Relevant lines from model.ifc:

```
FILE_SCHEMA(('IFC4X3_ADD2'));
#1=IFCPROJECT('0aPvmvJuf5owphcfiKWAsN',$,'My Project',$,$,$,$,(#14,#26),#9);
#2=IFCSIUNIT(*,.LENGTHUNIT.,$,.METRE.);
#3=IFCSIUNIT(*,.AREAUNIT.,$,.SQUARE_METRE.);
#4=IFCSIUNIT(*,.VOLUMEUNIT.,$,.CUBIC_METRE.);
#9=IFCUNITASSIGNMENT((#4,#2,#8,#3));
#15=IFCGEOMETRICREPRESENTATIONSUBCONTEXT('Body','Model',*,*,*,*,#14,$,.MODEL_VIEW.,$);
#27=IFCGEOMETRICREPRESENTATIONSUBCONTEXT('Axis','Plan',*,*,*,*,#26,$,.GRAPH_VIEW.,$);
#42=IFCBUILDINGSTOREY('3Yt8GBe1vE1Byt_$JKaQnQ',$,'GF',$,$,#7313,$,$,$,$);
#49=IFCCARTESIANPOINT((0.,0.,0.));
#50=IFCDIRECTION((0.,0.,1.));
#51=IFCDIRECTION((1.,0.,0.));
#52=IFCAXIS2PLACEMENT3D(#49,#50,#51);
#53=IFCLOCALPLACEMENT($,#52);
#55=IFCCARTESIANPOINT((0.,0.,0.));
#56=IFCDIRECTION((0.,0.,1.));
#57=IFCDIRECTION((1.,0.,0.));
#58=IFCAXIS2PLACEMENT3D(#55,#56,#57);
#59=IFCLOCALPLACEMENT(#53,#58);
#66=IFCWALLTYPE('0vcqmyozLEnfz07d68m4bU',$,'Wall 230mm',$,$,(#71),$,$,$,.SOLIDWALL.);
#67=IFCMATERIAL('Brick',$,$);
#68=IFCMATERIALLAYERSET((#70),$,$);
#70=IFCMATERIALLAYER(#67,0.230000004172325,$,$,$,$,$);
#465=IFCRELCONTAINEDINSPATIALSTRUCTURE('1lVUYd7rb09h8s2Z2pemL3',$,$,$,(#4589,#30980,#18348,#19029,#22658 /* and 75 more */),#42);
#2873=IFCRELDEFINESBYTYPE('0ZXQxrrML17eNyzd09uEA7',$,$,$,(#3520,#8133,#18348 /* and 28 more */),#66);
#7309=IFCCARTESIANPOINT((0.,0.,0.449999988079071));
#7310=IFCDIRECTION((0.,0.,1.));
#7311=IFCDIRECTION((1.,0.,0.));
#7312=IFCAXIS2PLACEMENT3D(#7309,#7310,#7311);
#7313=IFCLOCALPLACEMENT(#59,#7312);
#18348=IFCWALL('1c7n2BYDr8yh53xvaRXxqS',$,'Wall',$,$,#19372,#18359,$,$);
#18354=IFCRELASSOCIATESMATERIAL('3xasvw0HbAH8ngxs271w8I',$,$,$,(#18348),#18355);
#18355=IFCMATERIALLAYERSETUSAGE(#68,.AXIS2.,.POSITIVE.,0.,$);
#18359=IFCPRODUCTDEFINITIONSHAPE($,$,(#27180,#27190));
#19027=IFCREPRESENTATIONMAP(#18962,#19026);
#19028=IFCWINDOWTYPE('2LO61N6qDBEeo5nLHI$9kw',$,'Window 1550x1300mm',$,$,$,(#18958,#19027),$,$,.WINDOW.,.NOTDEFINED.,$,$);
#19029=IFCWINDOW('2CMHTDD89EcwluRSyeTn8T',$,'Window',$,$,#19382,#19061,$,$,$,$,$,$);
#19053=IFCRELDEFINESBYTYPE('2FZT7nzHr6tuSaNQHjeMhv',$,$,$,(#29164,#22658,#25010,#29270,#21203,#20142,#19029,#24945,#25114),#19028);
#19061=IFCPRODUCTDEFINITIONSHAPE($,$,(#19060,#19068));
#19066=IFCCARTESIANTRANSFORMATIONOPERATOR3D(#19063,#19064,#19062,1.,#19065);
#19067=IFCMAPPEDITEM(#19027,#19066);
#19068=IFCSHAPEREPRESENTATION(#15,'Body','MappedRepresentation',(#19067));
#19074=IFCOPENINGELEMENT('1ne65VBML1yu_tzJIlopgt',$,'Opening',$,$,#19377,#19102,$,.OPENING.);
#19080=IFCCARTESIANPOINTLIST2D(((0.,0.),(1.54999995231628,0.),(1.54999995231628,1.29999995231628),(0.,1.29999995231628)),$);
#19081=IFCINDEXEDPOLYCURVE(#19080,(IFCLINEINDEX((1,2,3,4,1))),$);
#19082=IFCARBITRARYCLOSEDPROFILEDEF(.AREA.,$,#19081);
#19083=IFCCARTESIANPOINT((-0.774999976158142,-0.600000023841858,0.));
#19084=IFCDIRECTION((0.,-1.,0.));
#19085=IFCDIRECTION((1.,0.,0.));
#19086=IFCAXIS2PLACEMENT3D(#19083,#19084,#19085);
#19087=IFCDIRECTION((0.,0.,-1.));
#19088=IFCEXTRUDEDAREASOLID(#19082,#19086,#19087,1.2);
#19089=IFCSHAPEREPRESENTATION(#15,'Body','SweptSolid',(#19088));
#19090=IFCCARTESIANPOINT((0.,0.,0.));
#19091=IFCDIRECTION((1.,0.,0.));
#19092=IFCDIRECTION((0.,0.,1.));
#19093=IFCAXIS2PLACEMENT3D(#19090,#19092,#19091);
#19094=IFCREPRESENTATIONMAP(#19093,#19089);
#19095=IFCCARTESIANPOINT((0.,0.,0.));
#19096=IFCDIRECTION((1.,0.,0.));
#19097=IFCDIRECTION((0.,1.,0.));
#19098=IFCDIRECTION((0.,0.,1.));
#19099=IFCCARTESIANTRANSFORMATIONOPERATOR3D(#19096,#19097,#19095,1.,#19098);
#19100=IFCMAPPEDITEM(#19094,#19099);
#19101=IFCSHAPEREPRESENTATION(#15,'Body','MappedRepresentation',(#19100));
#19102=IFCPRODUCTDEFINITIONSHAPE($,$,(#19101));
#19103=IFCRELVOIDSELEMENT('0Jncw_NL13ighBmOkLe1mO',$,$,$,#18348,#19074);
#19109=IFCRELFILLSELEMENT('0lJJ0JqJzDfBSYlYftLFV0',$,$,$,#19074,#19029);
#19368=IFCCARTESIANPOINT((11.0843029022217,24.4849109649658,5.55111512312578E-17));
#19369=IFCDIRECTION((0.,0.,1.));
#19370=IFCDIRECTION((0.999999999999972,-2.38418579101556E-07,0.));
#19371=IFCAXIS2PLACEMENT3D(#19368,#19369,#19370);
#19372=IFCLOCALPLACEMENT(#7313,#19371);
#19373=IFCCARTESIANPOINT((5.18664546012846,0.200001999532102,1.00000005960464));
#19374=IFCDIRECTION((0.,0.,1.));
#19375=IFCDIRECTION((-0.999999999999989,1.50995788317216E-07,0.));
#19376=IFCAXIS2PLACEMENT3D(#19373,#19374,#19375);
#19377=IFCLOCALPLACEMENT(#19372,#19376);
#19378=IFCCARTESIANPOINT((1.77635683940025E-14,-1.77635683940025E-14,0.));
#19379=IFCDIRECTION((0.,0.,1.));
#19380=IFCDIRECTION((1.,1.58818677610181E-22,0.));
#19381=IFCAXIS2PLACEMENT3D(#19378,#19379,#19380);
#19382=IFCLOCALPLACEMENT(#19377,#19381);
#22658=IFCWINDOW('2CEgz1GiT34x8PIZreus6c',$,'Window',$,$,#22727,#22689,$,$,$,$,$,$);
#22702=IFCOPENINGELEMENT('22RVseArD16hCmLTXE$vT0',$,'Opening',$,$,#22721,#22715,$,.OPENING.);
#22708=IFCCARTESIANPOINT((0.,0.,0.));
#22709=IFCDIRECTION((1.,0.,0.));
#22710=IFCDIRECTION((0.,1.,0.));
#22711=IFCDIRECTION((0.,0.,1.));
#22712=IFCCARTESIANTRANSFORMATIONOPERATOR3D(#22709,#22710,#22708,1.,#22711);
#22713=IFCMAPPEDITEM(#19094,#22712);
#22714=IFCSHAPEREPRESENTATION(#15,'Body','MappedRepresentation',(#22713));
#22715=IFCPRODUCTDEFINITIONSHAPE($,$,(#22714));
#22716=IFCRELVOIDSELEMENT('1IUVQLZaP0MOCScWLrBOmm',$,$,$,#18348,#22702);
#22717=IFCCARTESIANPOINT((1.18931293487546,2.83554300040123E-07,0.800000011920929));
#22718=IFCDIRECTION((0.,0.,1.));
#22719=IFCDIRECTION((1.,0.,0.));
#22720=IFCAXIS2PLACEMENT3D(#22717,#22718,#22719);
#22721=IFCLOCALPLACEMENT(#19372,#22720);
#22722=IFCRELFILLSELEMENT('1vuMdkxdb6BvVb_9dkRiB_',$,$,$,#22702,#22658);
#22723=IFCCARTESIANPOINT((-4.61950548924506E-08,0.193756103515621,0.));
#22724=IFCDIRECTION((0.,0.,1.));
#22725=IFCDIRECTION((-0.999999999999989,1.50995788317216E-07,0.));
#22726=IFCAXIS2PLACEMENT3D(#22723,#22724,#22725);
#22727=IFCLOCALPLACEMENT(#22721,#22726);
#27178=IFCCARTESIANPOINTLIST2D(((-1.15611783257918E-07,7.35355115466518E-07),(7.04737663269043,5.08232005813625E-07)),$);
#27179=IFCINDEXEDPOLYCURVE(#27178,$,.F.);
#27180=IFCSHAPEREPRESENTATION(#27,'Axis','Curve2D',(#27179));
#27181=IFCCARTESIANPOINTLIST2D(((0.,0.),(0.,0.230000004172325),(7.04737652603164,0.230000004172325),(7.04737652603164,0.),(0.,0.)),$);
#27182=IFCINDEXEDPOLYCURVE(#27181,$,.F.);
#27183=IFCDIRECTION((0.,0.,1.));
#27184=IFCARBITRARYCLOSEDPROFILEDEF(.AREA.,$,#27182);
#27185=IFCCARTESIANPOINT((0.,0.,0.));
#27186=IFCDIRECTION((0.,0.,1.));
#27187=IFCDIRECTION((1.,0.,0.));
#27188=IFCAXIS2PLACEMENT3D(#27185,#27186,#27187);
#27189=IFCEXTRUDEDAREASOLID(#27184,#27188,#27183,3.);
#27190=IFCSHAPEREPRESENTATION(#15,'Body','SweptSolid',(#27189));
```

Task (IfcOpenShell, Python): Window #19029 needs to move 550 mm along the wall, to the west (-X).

```python
import ifcopenshell
import ifcopenshell.api.geometry
import ifcopenshell.util.placement
import ifcopenshell.util.unit

model = ifcopenshell.open("model.ifc")
unit_scale = ifcopenshell.util.unit.calculate_unit_scale(model)

window = model.by_id(19029)
opening = window.FillsVoids[0].RelatingOpeningElement
wall = opening.VoidsElements[0].RelatingBuildingElement

wall_matrix = ifcopenshell.util.placement.get_local_placement(wall.ObjectPlacement)
shift = wall_matrix[:3, 0] * -0.55 / unit_scale
before = ifcopenshell.util.placement.get_local_placement(window.ObjectPlacement)[:3, 3].copy()

# The window is placed relative to its opening, so it follows when the opening moves.
matrix = ifcopenshell.util.placement.get_local_placement(opening.ObjectPlacement)
matrix[:3, 3] += shift
ifcopenshell.api.geometry.edit_object_placement(
    model, product=opening, matrix=matrix, is_si=False, should_transform_children=True
)

after = ifcopenshell.util.placement.get_local_placement(window.ObjectPlacement)[:3, 3]
print("window moved by", (after - before).round(3) + 0.0)

model.write("model_updated.ifc")
```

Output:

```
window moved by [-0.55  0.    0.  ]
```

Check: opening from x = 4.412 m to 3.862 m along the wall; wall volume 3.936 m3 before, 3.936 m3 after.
